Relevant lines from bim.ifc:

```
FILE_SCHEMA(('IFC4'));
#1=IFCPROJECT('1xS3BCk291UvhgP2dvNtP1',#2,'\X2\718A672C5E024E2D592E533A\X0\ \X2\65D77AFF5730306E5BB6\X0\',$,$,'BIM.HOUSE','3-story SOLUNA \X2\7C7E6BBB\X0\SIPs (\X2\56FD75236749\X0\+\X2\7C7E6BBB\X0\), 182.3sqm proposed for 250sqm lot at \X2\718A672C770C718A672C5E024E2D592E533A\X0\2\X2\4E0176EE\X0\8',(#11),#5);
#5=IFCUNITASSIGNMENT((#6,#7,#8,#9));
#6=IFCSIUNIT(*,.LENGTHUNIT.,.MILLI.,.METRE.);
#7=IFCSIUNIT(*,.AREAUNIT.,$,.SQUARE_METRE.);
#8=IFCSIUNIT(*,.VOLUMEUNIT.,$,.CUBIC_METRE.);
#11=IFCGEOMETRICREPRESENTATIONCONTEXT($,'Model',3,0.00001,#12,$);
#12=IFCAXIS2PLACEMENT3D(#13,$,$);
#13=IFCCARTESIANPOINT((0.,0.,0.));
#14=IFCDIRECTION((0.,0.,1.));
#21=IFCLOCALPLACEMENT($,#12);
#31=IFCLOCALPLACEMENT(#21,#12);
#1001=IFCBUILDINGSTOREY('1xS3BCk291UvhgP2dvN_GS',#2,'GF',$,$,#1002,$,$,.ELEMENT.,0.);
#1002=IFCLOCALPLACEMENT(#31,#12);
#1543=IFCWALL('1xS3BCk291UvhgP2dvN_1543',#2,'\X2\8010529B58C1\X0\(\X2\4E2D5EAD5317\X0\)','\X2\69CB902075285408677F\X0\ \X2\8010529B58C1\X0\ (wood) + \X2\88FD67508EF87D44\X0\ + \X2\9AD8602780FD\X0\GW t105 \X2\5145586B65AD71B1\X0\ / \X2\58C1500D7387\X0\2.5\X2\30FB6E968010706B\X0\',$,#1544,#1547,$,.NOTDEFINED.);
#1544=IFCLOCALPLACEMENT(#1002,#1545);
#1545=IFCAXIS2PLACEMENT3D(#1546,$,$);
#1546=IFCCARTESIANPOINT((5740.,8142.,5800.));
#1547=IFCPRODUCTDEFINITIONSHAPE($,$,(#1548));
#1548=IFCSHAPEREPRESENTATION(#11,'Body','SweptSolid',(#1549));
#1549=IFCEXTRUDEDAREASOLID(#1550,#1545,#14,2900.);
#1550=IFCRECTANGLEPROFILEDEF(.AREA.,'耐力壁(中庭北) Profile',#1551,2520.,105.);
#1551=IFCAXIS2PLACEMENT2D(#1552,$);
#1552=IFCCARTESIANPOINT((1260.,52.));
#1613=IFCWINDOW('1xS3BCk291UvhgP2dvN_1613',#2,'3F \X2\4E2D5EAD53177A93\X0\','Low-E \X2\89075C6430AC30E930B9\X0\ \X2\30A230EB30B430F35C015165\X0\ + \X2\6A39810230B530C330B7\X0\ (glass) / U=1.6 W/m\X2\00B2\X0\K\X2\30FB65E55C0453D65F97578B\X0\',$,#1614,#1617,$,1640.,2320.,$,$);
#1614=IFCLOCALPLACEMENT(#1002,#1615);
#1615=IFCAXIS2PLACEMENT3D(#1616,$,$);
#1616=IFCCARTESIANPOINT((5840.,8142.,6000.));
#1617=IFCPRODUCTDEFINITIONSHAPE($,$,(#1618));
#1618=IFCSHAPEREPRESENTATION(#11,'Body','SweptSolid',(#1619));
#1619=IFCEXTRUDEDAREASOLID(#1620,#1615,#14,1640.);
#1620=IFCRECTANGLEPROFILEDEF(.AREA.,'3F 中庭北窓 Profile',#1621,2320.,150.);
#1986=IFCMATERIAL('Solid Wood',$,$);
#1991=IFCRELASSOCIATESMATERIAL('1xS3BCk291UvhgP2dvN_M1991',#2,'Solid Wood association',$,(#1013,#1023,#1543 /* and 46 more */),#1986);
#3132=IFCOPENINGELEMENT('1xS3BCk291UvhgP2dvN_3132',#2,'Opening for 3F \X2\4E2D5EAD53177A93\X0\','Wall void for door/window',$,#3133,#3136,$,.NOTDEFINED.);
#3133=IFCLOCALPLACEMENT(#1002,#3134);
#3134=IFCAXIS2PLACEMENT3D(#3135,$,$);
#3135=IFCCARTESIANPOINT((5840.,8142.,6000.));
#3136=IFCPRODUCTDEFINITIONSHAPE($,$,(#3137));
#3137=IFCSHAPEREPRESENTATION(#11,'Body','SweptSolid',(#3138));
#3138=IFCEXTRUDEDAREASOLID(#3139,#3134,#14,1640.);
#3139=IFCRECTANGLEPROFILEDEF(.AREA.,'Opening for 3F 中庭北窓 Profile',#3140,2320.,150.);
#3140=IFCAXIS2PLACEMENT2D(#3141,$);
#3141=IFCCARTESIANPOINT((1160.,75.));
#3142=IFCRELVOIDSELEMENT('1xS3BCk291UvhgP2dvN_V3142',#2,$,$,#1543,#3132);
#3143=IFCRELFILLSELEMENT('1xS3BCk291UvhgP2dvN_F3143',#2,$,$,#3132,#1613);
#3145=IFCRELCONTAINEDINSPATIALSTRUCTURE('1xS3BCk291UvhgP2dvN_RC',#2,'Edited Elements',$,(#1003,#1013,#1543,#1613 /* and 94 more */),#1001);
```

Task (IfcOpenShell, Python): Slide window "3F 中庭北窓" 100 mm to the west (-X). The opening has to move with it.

```python
import ifcopenshell
import ifcopenshell.api.geometry
import ifcopenshell.util.placement

model = ifcopenshell.open("bim.ifc")

window = model.by_id(1613)
opening = window.FillsVoids[0].RelatingOpeningElement
wall = opening.VoidsElements[0].RelatingBuildingElement

wall_matrix = ifcopenshell.util.placement.get_local_placement(wall.ObjectPlacement)
shift = wall_matrix[:3, 0] * -100.0
before = ifcopenshell.util.placement.get_local_placement(window.ObjectPlacement)[:3, 3].copy()

# The window is not placed relative to its opening, so move both.
for product in (opening, window):
    matrix = ifcopenshell.util.placement.get_local_placement(product.ObjectPlacement)
    matrix[:3, 3] += shift
    ifcopenshell.api.geometry.edit_object_placement(model, product=product, matrix=matrix, is_si=False)

after = ifcopenshell.util.placement.get_local_placement(window.ObjectPlacement)[:3, 3]
print("window moved by", (after - before).round(3) + 0.0)

model.write("bim_rev.ifc")
```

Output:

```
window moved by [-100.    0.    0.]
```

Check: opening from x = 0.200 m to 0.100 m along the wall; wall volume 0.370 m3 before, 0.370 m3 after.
